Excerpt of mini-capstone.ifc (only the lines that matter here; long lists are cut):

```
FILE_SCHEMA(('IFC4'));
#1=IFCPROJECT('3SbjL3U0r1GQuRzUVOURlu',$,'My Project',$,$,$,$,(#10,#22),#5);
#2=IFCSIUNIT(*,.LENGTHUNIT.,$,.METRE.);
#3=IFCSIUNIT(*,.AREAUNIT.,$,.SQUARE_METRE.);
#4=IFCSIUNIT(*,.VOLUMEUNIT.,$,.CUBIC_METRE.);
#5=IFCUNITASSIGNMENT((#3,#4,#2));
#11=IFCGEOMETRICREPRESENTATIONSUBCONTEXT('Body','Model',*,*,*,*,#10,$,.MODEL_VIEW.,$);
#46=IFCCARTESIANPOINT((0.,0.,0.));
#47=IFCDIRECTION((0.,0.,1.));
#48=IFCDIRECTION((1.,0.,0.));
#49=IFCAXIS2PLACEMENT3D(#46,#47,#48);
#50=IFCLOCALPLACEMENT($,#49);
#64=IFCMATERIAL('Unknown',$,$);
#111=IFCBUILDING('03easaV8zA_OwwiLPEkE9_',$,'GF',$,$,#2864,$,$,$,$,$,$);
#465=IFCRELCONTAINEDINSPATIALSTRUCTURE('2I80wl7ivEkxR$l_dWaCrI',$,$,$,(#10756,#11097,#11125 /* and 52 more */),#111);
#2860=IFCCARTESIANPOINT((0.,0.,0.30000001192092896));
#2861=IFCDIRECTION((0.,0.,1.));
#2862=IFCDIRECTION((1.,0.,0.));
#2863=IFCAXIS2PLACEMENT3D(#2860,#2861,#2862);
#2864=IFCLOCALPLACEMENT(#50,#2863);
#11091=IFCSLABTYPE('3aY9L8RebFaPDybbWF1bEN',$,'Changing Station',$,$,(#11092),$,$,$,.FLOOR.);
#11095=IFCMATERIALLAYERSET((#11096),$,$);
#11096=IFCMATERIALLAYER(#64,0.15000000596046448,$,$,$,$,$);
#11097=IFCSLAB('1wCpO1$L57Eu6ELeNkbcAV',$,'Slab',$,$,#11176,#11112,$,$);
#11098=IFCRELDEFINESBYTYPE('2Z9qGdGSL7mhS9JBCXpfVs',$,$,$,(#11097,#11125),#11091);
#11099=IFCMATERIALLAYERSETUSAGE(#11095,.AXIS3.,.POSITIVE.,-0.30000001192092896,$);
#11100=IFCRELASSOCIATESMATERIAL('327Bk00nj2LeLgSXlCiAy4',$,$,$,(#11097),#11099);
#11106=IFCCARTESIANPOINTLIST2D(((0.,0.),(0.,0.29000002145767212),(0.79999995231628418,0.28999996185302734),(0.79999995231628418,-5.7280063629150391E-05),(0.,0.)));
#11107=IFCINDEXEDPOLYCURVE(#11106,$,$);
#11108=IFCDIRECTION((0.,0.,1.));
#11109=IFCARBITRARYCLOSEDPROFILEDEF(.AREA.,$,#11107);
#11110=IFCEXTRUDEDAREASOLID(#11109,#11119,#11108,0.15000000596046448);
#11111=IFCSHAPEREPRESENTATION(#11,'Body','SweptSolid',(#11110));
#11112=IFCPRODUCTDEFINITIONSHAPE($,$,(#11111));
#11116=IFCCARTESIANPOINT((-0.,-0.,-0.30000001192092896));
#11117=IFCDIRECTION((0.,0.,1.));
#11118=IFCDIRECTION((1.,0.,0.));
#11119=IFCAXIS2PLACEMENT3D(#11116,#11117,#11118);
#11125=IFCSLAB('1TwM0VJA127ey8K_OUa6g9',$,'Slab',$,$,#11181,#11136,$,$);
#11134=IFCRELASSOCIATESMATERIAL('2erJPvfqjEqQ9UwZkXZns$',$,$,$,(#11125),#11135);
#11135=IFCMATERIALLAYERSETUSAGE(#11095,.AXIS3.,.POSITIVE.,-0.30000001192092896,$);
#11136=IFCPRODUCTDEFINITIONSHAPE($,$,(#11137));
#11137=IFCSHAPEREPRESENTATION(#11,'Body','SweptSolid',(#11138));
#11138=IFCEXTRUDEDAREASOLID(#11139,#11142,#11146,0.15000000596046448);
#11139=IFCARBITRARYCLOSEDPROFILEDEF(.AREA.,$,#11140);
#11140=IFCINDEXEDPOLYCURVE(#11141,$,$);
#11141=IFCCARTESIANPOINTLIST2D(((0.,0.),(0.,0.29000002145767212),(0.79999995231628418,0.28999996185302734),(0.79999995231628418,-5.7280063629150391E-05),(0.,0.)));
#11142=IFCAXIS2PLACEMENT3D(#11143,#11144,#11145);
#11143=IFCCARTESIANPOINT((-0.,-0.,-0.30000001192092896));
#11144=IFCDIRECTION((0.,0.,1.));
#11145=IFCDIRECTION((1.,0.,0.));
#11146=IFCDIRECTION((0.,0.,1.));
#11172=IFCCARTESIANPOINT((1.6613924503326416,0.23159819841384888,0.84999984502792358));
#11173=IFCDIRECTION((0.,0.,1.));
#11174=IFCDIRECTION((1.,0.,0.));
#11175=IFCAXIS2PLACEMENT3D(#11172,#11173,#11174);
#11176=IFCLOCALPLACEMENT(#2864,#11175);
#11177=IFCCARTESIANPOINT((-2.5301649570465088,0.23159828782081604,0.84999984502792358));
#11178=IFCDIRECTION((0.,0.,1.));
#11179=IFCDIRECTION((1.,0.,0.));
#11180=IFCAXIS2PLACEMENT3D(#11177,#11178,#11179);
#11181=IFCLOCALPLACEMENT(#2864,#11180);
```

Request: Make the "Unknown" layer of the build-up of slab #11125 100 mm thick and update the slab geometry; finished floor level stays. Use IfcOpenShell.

```python
import ifcopenshell
import ifcopenshell.util.element
import ifcopenshell.util.representation
import ifcopenshell.util.unit

model = ifcopenshell.open("mini-capstone.ifc")
unit_scale = ifcopenshell.util.unit.calculate_unit_scale(model)

layer_set = model.by_id(11095)
layer = next(l for l in layer_set.MaterialLayers if l.Material and l.Material.Name == "Unknown")
change = 0.1 / unit_scale - layer.LayerThickness
layer.LayerThickness += change

# The layer set is shared, so every slab that uses it gets the new thickness.
slabs = [e for e in ifcopenshell.util.element.get_elements_by_material(model, layer_set) if e.is_a("IfcSlab")]
for slab in sorted(slabs, key=lambda e: e.id()):
    body = ifcopenshell.util.representation.get_representation(slab, "Model", "Body")
    solid = body.Items[0]
    old_depth = solid.Depth
    solid.Depth += change
    # Extruded upwards: lower the start of the extrusion so the top stays.
    x, y, z = solid.Position.Location.Coordinates
    solid.Position.Location = model.createIfcCartesianPoint((x, y, z - change))
    print(slab.id(), f"{old_depth:g} -> {solid.Depth:g}")

# The layers are counted up from the underside, which has moved.
for usage in {ifcopenshell.util.element.get_material(slab) for slab in slabs}:
    usage.OffsetFromReferenceLine -= change

model.write("mini-capstone_v2.ifc")
```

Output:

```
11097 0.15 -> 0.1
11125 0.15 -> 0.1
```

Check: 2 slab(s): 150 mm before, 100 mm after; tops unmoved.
